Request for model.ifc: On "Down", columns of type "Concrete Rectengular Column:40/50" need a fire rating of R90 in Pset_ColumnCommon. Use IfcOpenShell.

First a look at what the model holds.

```python
import ifcopenshell
import ifcopenshell.util.element

model = ifcopenshell.open("model.ifc")
print(model.schema)
storey = next(s for s in model.by_type("IfcBuildingStorey") if s.Name == "Down")
columns = [e for e in ifcopenshell.util.element.get_decomposition(storey) if e.is_a("IfcColumn")]
seen = {}
for e in columns:
    element_type = ifcopenshell.util.element.get_type(e)
    key = (element_type.Name if element_type != e and element_type else None, ifcopenshell.util.element.get_pset(e, "Pset_ColumnCommon", "FireRating"))
    seen[key] = seen.get(key, 0) + 1
for (name, value), count in sorted(seen.items(), key=str):
    print(count, "x", name, "|", value)
```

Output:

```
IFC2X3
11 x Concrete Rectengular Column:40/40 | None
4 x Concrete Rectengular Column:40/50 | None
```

```python
import ifcopenshell
import ifcopenshell.api.pset
import ifcopenshell.util.element

model = ifcopenshell.open("model.ifc")

storey = next(s for s in model.by_type("IfcBuildingStorey") if s.Name == "Down")
columns = [e for e in ifcopenshell.util.element.get_decomposition(storey) if e.is_a("IfcColumn")]

count = 0
for e in columns:
    element_type = ifcopenshell.util.element.get_type(e)
    if element_type in (None, e) or element_type.Name != "Concrete Rectengular Column:40/50":
        continue
    # add_pset returns the element's existing set when there is one.
    pset = ifcopenshell.api.pset.add_pset(model, product=e, name="Pset_ColumnCommon")
    ifcopenshell.api.pset.edit_pset(model, pset=pset, properties={"FireRating": "R90"})
    count += 1

print(count, "columns updated")

model.write("model-out.ifc")
```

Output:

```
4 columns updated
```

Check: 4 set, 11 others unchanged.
